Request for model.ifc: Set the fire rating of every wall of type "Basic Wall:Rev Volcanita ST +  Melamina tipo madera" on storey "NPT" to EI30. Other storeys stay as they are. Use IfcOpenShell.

First a look at what the model holds.

```python
import ifcopenshell
import ifcopenshell.util.element

model = ifcopenshell.open("model.ifc")
print(model.schema)
storey = next(s for s in model.by_type("IfcBuildingStorey") if s.Name == "NPT")
walls = [e for e in ifcopenshell.util.element.get_decomposition(storey) if e.is_a("IfcWall")]
seen = {}
for e in walls:
    element_type = ifcopenshell.util.element.get_type(e)
    key = (element_type.Name if element_type != e and element_type else None, ifcopenshell.util.element.get_pset(e, "Pset_WallCommon", "FireRating"))
    seen[key] = seen.get(key, 0) + 1
for (name, value), count in sorted(seen.items(), key=str):
    print(count, "x", name, "|", value)
```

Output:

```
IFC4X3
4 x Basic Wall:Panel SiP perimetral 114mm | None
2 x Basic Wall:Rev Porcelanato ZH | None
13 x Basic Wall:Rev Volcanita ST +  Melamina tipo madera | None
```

```python
import ifcopenshell
import ifcopenshell.api.pset
import ifcopenshell.util.element

model = ifcopenshell.open("model.ifc")

storey = next(s for s in model.by_type("IfcBuildingStorey") if s.Name == "NPT")
walls = [e for e in ifcopenshell.util.element.get_decomposition(storey) if e.is_a("IfcWall")]

count = 0
for e in walls:
    element_type = ifcopenshell.util.element.get_type(e)
    if element_type in (None, e) or element_type.Name != "Basic Wall:Rev Volcanita ST +  Melamina tipo madera":
        continue
    # add_pset returns the element's existing set when there is one.
    pset = ifcopenshell.api.pset.add_pset(model, product=e, name="Pset_WallCommon")
    ifcopenshell.api.pset.edit_pset(model, pset=pset, properties={"FireRating": "EI30"})
    count += 1

print(count, "walls updated")

model.write("model_rev.ifc")
```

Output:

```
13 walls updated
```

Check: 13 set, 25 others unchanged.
